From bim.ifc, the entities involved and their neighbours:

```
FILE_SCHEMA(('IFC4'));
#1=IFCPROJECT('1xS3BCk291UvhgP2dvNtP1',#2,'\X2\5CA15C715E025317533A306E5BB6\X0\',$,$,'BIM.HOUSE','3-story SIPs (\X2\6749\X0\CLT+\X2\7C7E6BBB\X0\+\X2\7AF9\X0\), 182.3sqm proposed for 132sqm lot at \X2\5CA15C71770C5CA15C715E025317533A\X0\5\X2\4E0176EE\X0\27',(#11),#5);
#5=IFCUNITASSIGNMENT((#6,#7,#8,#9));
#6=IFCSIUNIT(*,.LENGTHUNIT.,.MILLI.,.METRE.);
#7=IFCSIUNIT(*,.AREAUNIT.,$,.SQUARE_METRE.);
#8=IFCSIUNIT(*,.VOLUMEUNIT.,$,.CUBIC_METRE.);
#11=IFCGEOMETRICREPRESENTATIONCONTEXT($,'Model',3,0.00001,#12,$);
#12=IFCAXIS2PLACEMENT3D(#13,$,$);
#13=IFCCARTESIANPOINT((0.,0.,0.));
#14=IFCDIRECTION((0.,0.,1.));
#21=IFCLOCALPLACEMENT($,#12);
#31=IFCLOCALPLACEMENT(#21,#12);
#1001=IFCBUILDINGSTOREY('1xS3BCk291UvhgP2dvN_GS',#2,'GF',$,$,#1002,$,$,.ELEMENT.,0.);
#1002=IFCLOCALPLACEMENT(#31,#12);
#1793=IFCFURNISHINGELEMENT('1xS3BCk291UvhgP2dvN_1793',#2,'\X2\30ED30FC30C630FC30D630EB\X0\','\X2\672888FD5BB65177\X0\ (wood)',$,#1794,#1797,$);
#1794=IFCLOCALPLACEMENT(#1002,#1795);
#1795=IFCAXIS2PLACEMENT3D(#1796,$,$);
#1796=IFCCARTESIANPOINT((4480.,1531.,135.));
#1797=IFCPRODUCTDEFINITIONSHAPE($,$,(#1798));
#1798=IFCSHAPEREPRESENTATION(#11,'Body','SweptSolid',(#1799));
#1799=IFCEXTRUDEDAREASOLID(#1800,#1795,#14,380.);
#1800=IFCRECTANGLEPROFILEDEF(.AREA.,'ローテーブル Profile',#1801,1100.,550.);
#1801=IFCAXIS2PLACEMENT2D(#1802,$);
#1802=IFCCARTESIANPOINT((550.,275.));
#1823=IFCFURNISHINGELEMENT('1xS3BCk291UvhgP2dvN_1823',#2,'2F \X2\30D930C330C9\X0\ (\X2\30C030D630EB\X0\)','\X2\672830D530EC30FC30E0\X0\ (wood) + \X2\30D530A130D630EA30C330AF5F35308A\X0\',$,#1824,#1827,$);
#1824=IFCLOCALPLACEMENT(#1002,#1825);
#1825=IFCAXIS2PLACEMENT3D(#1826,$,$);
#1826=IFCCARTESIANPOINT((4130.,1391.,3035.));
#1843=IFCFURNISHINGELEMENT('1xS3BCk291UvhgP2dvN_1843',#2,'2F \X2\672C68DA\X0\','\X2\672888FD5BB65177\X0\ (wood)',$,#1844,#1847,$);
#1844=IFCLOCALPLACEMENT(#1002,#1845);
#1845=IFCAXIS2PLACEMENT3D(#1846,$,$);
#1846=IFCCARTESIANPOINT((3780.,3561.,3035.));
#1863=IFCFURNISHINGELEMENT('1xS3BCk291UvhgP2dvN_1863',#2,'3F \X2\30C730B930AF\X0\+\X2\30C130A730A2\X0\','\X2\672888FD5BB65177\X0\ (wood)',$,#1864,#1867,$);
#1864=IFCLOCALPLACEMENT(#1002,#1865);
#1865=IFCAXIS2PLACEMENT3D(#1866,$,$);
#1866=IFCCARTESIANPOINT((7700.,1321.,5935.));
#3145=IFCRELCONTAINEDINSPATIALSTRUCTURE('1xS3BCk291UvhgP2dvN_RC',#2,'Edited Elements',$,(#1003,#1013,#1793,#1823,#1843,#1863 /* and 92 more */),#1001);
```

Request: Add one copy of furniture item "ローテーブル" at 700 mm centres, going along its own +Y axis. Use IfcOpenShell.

```python
import ifcopenshell
import ifcopenshell.api.geometry
import ifcopenshell.api.root
import ifcopenshell.util.element
import ifcopenshell.util.placement

model = ifcopenshell.open("bim.ifc")


def reuse_history(source, copy):
    """copy_class also copies each property set's owner history, people and application; keep the originals."""
    for rel in copy.IsDefinedBy:
        if rel.is_a("IfcRelDefinesByProperties") and (history := rel.RelatingPropertyDefinition.OwnerHistory):
            rel.RelatingPropertyDefinition.OwnerHistory = source.OwnerHistory
            ifcopenshell.util.element.remove_deep2(model, history)


source = model.by_id(1793)
base = ifcopenshell.util.placement.get_local_placement(source.ObjectPlacement)
step = base[:3, 1] * 700.0

for i in range(1, 2):
    copy = ifcopenshell.api.root.copy_class(model, product=source)
    copy.Representation = ifcopenshell.util.element.copy_deep(
        model, source.Representation, exclude=["IfcGeometricRepresentationContext", "IfcRepresentationMap"]
    )
    reuse_history(source, copy)
    matrix = base.copy()
    matrix[:3, 3] += i * step
    print("added at", matrix[:3, 3].round(3) + 0.0)
    ifcopenshell.api.geometry.edit_object_placement(model, product=copy, matrix=matrix, is_si=False)

model.write("bim_rev.ifc")
```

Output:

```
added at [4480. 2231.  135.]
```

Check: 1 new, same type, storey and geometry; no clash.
